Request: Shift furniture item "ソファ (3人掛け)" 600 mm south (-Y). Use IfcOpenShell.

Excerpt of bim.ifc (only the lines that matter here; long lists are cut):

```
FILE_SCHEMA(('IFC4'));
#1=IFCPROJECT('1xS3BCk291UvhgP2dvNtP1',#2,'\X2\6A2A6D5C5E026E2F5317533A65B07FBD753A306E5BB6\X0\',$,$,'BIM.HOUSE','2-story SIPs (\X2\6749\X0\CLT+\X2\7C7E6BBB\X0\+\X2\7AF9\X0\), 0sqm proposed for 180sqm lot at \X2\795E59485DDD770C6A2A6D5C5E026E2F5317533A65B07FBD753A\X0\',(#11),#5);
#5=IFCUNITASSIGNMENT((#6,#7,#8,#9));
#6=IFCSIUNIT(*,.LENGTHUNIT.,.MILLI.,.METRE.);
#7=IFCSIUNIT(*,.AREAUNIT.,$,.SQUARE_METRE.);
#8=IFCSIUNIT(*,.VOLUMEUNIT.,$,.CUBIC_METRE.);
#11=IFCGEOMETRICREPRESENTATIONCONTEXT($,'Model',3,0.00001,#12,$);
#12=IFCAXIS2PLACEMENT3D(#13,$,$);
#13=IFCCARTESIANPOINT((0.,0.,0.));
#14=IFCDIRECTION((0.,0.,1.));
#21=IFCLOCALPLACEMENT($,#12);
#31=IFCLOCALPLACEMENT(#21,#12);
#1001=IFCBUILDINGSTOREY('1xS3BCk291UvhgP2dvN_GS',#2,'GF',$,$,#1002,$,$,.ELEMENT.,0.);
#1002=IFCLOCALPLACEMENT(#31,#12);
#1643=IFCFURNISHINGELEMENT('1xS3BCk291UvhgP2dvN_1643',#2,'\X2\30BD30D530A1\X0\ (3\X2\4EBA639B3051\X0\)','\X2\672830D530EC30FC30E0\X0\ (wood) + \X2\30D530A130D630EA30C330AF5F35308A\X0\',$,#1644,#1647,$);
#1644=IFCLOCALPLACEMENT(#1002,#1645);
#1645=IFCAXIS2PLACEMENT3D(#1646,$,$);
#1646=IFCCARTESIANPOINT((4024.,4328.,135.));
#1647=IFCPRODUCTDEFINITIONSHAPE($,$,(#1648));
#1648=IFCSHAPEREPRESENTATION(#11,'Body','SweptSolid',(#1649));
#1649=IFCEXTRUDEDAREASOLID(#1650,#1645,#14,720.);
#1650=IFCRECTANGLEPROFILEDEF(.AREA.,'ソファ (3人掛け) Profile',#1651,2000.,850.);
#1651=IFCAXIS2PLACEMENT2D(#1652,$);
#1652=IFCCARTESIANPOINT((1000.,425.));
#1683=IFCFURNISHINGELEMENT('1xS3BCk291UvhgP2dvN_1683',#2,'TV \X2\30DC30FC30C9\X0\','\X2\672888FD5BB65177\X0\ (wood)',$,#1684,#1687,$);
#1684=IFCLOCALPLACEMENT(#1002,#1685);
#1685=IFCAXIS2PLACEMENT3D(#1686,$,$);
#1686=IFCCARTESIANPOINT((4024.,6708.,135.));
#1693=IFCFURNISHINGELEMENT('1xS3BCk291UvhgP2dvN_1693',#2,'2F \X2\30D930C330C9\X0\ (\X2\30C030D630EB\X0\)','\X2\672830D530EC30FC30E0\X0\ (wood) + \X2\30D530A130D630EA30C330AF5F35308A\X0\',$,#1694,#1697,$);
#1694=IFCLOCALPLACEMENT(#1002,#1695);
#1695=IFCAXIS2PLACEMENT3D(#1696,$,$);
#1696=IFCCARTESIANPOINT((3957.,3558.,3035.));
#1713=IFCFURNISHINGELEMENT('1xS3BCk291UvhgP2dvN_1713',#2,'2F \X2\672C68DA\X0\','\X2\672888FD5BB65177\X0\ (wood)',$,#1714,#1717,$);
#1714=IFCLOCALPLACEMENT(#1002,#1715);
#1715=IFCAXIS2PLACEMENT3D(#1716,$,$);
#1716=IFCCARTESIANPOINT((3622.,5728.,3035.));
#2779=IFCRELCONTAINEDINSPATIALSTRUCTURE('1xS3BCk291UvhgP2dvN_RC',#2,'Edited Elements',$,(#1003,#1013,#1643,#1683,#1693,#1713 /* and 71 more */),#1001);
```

```python
import ifcopenshell
import ifcopenshell.api.geometry
import ifcopenshell.util.placement
import ifcopenshell.util.unit

model = ifcopenshell.open("bim.ifc")
unit_scale = ifcopenshell.util.unit.calculate_unit_scale(model)

item = model.by_guid("1xS3BCk291UvhgP2dvN_1643")
matrix = ifcopenshell.util.placement.get_local_placement(item.ObjectPlacement)
matrix[1, 3] -= 0.6 / unit_scale
ifcopenshell.api.geometry.edit_object_placement(model, product=item, matrix=matrix, is_si=False)

print(ifcopenshell.util.placement.get_local_placement(item.ObjectPlacement).round(3) + 0.0)

model.write("bim_rev.ifc")
```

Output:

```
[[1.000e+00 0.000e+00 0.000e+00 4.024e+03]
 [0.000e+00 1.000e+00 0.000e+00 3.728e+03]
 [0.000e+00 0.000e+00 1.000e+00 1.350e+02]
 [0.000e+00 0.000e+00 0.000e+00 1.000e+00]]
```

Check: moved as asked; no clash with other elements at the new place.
